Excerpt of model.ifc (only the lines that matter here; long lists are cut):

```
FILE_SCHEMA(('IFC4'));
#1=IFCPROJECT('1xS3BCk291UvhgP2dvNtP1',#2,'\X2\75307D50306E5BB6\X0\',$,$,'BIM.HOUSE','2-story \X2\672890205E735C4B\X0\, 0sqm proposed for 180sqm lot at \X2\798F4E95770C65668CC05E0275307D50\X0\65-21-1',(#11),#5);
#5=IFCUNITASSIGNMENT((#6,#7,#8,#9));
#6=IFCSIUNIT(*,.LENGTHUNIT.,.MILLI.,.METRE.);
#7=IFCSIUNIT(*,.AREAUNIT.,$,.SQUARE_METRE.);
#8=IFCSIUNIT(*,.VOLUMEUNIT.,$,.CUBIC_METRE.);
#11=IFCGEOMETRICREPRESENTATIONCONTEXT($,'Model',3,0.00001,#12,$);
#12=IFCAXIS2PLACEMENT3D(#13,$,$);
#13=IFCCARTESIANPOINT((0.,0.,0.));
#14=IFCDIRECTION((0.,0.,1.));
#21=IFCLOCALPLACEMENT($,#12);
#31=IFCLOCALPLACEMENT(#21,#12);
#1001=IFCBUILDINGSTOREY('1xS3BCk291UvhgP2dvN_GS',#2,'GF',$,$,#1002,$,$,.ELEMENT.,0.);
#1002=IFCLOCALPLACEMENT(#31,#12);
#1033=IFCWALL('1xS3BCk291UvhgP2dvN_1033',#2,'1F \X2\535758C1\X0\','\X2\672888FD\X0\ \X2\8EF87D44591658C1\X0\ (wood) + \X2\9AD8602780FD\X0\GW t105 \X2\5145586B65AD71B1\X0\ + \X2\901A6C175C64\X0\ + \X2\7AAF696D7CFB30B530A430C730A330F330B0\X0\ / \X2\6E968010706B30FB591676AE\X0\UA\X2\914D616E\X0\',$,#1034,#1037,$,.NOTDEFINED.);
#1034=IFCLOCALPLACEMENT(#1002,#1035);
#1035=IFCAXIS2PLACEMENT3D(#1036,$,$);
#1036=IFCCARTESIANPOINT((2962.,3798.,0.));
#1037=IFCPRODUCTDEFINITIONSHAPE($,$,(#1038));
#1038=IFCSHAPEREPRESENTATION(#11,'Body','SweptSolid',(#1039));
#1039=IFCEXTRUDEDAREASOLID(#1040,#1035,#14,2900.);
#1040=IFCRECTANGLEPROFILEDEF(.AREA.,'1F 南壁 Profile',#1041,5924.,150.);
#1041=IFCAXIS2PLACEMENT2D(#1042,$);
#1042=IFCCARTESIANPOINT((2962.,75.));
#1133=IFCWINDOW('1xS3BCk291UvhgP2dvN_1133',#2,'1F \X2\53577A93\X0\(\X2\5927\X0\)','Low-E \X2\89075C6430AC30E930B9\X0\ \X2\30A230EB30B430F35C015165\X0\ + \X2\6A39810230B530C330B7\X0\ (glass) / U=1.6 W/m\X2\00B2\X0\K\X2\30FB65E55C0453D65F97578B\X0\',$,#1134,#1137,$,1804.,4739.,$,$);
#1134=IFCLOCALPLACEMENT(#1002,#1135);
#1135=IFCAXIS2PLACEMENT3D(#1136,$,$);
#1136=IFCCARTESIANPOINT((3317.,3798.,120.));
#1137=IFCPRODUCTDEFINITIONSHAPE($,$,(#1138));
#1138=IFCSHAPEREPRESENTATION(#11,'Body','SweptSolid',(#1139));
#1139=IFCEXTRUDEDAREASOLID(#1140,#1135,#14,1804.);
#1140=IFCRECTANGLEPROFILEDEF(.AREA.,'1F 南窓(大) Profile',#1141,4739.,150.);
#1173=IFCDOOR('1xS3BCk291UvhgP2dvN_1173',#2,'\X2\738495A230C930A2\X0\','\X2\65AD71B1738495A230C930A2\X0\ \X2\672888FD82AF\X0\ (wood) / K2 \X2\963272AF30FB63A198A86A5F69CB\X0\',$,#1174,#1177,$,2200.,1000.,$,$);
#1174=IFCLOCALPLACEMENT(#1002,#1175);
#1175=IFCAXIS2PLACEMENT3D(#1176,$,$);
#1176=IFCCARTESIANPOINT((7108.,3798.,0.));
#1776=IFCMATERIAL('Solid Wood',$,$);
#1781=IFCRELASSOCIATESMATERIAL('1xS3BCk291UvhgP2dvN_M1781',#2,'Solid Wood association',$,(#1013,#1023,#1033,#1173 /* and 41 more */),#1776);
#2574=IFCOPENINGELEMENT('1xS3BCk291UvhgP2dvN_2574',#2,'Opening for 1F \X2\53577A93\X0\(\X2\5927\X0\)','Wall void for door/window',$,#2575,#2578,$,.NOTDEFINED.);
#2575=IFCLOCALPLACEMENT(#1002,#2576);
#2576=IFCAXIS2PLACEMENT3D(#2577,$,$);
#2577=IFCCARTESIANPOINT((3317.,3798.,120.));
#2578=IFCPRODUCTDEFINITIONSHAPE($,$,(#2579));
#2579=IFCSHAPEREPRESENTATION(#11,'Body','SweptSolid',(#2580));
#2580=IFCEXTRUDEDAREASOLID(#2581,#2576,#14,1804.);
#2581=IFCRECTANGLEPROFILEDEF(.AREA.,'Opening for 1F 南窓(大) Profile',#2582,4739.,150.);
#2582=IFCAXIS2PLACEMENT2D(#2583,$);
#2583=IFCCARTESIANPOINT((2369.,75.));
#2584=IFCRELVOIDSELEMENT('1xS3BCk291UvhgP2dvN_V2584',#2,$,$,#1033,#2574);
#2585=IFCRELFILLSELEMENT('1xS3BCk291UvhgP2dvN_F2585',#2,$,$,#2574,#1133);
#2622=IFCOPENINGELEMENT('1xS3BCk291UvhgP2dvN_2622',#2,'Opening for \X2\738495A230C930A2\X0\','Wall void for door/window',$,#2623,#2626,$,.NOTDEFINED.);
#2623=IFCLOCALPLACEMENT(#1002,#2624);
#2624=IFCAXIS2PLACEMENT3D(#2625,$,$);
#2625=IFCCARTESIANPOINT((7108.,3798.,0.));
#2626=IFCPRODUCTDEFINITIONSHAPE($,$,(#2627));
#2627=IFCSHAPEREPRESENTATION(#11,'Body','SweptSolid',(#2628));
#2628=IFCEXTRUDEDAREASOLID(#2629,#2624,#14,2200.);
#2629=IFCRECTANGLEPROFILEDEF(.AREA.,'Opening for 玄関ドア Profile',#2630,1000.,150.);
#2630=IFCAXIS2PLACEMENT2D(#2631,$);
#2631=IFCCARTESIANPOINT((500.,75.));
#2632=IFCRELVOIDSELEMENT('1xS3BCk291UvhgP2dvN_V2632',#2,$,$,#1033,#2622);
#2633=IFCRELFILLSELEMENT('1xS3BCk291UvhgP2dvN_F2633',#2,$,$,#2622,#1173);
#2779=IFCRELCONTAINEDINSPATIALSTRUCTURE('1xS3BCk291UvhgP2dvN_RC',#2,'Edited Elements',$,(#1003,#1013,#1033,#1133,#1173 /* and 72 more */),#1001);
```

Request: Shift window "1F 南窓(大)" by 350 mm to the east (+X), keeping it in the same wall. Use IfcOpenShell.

```python
import ifcopenshell
import ifcopenshell.api.geometry
import ifcopenshell.util.placement
import ifcopenshell.util.unit

model = ifcopenshell.open("model.ifc")
unit_scale = ifcopenshell.util.unit.calculate_unit_scale(model)

window = model.by_id(1133)
opening = window.FillsVoids[0].RelatingOpeningElement
wall = opening.VoidsElements[0].RelatingBuildingElement

wall_matrix = ifcopenshell.util.placement.get_local_placement(wall.ObjectPlacement)
shift = wall_matrix[:3, 0] * 0.35 / unit_scale
before = ifcopenshell.util.placement.get_local_placement(window.ObjectPlacement)[:3, 3].copy()

# The window is not placed relative to its opening, so move both.
for product in (opening, window):
    matrix = ifcopenshell.util.placement.get_local_placement(product.ObjectPlacement)
    matrix[:3, 3] += shift
    ifcopenshell.api.geometry.edit_object_placement(model, product=product, matrix=matrix, is_si=False)

after = ifcopenshell.util.placement.get_local_placement(window.ObjectPlacement)[:3, 3]
print("window moved by", (after - before).round(3) + 0.0)

model.write("model_updated.ifc")
```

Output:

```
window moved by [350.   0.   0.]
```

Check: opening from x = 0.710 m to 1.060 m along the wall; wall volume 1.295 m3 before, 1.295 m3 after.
